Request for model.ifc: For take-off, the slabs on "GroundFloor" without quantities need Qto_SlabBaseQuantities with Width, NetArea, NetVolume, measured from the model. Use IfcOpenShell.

First a look at what the model holds.

```python
import ifcopenshell
import ifcopenshell.util.element
import ifcopenshell.util.unit

model = ifcopenshell.open("model.ifc")
print(model.schema)
for unit_type in ("LENGTHUNIT", "AREAUNIT", "VOLUMEUNIT"):
    print(unit_type, ifcopenshell.util.unit.calculate_unit_scale(model, unit_type))
storey = next(s for s in model.by_type("IfcBuildingStorey") if s.Name == "GroundFloor")
slabs = [e for e in ifcopenshell.util.element.get_decomposition(storey) if e.is_a("IfcSlab")]
for e in sorted(slabs, key=lambda e: e.id()):
    print(e.id(), e.is_a(), e.Name, list(ifcopenshell.util.element.get_psets(e, qtos_only=True)), sep=" | ")
```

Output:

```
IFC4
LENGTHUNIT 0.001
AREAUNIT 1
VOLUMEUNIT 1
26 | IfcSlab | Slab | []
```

```python
import ifcopenshell
import ifcopenshell.api.pset
import ifcopenshell.geom
import ifcopenshell.util.element
import ifcopenshell.util.shape
import ifcopenshell.util.unit

model = ifcopenshell.open("model.ifc")
unit_scale = ifcopenshell.util.unit.calculate_unit_scale(model)
area_scale = ifcopenshell.util.unit.calculate_unit_scale(model, "AREAUNIT")
volume_scale = ifcopenshell.util.unit.calculate_unit_scale(model, "VOLUMEUNIT")
settings = ifcopenshell.geom.settings()

storey = next(s for s in model.by_type("IfcBuildingStorey") if s.Name == "GroundFloor")
slabs = [e for e in ifcopenshell.util.element.get_decomposition(storey) if e.is_a("IfcSlab")]

for e in sorted(slabs, key=lambda e: e.id()):
    if ifcopenshell.util.element.get_psets(e, qtos_only=True, should_inherit=False):
        continue
    # Geometry comes back in metres, in the element's own axes.
    shape = ifcopenshell.geom.create_shape(settings, e)
    values = {
        "Width": ifcopenshell.util.shape.get_z(shape.geometry) / unit_scale,
        "NetArea": ifcopenshell.util.shape.get_footprint_area(shape.geometry) / area_scale,
        "NetVolume": ifcopenshell.util.shape.get_volume(shape.geometry) / volume_scale,
    }
    qto = ifcopenshell.api.pset.add_qto(model, product=e, name="Qto_SlabBaseQuantities")
    ifcopenshell.api.pset.edit_qto(model, qto=qto, properties=values)
    print(e.id(), {k: round(v, 3) for k, v in values.items()})

model.write("model_updated.ifc")
```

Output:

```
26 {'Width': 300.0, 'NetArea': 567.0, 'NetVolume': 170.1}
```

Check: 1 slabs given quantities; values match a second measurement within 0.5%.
